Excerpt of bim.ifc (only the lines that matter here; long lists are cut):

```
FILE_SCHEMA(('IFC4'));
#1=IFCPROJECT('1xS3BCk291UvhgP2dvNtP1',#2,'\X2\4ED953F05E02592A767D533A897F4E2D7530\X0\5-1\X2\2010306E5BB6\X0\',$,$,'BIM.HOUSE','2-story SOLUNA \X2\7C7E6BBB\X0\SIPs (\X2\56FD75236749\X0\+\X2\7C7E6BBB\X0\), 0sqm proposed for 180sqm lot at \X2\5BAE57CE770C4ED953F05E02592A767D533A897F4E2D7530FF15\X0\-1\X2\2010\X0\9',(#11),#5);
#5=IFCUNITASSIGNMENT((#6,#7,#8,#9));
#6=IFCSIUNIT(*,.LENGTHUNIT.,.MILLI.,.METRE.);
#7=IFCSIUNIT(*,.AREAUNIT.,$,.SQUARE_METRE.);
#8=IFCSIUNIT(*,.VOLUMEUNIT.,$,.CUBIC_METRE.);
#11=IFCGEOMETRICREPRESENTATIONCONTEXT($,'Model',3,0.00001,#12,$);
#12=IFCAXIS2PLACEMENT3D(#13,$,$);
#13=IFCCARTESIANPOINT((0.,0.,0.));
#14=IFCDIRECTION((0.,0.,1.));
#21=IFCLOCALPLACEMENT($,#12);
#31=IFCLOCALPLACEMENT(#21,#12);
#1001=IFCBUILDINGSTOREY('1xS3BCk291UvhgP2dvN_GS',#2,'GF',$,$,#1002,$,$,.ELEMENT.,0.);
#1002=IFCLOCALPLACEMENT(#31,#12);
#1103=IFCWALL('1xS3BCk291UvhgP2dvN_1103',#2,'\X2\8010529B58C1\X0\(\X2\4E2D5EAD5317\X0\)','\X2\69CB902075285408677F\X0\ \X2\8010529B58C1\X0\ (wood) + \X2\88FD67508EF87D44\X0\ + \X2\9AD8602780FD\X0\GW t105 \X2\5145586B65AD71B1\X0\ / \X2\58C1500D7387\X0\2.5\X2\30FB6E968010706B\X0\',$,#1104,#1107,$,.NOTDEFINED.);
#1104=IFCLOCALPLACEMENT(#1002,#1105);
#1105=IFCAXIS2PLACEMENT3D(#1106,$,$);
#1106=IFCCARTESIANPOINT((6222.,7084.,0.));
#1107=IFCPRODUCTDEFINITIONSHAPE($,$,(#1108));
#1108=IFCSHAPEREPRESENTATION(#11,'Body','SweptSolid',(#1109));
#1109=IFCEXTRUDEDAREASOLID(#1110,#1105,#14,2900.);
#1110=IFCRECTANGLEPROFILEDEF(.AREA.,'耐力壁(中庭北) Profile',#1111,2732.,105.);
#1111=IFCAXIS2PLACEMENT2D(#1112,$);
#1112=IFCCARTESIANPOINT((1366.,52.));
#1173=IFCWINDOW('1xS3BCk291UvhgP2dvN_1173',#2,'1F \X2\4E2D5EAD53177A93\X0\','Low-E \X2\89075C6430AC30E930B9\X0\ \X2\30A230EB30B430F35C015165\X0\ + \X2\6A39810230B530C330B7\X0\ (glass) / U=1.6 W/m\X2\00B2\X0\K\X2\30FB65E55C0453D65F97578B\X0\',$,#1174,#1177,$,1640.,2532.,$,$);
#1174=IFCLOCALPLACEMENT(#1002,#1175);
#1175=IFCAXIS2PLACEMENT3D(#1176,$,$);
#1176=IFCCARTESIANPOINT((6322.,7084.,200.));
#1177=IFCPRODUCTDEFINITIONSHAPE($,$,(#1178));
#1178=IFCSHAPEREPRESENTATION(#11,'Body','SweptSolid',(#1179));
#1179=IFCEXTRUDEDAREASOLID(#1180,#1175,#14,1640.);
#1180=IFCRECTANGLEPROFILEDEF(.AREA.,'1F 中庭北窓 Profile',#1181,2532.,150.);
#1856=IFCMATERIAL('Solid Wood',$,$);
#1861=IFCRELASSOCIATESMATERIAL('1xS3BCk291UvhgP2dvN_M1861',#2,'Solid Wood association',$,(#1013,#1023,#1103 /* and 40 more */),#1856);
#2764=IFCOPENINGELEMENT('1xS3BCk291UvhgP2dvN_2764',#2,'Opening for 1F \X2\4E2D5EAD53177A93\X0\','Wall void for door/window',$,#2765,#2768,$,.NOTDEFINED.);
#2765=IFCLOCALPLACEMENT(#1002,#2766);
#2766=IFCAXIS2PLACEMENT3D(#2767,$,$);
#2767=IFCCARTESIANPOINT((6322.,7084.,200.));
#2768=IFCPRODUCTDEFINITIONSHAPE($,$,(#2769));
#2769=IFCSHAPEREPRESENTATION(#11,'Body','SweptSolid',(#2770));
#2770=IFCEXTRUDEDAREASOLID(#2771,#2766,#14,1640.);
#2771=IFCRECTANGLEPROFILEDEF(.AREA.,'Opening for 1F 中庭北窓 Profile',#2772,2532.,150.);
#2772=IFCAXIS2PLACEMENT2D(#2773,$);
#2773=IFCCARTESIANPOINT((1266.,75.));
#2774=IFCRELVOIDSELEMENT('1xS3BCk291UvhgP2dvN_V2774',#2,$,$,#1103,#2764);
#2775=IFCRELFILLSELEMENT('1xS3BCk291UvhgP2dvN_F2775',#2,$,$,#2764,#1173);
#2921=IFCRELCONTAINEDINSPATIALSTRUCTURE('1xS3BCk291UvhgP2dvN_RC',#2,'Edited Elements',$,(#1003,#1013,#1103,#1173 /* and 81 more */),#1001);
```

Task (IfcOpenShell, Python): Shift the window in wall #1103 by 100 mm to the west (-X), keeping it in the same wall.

```python
import ifcopenshell
import ifcopenshell.api.geometry
import ifcopenshell.util.placement

model = ifcopenshell.open("bim.ifc")

window = model.by_guid("1xS3BCk291UvhgP2dvN_1173")
opening = window.FillsVoids[0].RelatingOpeningElement
wall = opening.VoidsElements[0].RelatingBuildingElement

wall_matrix = ifcopenshell.util.placement.get_local_placement(wall.ObjectPlacement)
shift = wall_matrix[:3, 0] * -100.0
before = ifcopenshell.util.placement.get_local_placement(window.ObjectPlacement)[:3, 3].copy()

# The window is not placed relative to its opening, so move both.
for product in (opening, window):
    matrix = ifcopenshell.util.placement.get_local_placement(product.ObjectPlacement)
    matrix[:3, 3] += shift
    ifcopenshell.api.geometry.edit_object_placement(model, product=product, matrix=matrix, is_si=False)

after = ifcopenshell.util.placement.get_local_placement(window.ObjectPlacement)[:3, 3]
print("window moved by", (after - before).round(3) + 0.0)

model.write("bim_edited.ifc")
```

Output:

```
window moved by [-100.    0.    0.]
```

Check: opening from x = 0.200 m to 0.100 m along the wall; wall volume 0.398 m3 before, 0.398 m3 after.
